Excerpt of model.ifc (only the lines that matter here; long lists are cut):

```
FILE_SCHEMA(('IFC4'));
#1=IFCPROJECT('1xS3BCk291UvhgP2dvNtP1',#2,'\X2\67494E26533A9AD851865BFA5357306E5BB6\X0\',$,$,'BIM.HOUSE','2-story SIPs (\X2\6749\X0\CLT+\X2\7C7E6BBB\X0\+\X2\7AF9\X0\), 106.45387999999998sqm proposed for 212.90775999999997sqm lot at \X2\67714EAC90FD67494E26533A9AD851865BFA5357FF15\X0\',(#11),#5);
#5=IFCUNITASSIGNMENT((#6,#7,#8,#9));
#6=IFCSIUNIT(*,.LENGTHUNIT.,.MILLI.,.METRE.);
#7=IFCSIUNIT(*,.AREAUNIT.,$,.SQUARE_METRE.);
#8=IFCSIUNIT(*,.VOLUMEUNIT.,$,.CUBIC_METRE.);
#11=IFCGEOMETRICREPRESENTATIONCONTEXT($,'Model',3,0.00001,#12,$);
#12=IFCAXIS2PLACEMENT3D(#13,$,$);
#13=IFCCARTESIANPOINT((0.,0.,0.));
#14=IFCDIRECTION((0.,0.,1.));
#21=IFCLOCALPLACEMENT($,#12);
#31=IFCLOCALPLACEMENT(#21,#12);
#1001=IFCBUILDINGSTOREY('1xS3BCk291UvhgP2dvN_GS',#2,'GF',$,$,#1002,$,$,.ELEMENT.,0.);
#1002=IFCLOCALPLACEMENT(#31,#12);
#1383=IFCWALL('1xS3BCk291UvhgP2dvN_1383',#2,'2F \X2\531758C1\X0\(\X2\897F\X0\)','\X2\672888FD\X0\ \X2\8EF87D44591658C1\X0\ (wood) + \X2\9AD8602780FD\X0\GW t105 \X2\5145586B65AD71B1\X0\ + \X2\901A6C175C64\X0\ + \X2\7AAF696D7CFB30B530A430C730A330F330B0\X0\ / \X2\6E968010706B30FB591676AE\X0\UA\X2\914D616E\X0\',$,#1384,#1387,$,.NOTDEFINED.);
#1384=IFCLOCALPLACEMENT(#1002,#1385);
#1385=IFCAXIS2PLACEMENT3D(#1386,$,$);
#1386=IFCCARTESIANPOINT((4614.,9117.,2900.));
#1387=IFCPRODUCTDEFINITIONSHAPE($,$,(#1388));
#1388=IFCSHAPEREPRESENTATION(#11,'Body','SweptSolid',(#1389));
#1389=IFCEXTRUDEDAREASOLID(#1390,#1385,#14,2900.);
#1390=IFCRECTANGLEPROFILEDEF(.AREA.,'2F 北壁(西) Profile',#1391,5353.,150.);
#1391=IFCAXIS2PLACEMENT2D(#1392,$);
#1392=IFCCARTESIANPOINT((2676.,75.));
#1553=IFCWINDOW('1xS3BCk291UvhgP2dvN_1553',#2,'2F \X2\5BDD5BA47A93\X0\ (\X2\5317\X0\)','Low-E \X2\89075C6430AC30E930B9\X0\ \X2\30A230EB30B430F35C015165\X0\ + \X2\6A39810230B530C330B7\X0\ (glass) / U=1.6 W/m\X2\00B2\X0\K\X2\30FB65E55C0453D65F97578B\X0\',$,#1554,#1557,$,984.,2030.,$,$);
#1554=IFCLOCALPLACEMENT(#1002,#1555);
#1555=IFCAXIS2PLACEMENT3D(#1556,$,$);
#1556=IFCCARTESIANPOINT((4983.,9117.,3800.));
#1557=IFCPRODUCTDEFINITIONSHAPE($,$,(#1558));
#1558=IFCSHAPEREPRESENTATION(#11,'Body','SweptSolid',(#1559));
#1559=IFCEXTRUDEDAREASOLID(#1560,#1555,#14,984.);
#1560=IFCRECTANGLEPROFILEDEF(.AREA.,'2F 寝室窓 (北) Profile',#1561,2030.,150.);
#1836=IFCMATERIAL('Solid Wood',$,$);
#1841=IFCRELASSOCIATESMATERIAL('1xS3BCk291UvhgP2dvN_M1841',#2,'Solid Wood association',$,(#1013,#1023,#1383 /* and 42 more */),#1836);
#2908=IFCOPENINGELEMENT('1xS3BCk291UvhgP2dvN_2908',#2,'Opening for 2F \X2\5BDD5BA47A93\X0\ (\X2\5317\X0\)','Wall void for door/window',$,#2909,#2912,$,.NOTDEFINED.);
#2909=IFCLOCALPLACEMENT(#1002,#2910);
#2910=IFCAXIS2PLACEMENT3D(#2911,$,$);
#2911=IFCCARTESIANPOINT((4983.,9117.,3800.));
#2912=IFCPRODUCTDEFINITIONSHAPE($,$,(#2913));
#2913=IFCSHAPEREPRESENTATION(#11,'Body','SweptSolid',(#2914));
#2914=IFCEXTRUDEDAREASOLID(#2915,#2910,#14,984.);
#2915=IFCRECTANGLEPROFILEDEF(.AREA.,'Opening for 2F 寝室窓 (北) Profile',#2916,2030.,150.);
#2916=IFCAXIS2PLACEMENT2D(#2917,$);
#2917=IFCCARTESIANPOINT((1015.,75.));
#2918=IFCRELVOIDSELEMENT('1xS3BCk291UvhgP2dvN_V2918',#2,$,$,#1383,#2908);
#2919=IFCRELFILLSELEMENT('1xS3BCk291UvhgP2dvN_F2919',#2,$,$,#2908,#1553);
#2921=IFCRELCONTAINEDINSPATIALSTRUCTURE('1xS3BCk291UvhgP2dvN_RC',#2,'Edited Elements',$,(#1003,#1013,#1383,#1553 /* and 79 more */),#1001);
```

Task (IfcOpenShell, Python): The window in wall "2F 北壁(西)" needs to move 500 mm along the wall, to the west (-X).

```python
import ifcopenshell
import ifcopenshell.api.geometry
import ifcopenshell.util.placement
import ifcopenshell.util.unit

model = ifcopenshell.open("model.ifc")
unit_scale = ifcopenshell.util.unit.calculate_unit_scale(model)

window = model.by_guid("1xS3BCk291UvhgP2dvN_1553")
opening = window.FillsVoids[0].RelatingOpeningElement
wall = opening.VoidsElements[0].RelatingBuildingElement

wall_matrix = ifcopenshell.util.placement.get_local_placement(wall.ObjectPlacement)
shift = wall_matrix[:3, 0] * -0.5 / unit_scale
before = ifcopenshell.util.placement.get_local_placement(window.ObjectPlacement)[:3, 3].copy()

# The window is not placed relative to its opening, so move both.
for product in (opening, window):
    matrix = ifcopenshell.util.placement.get_local_placement(product.ObjectPlacement)
    matrix[:3, 3] += shift
    ifcopenshell.api.geometry.edit_object_placement(model, product=product, matrix=matrix, is_si=False)

after = ifcopenshell.util.placement.get_local_placement(window.ObjectPlacement)[:3, 3]
print("window moved by", (after - before).round(3) + 0.0)

model.write("model-out.ifc")
```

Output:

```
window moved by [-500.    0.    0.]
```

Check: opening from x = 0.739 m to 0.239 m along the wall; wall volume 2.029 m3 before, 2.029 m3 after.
